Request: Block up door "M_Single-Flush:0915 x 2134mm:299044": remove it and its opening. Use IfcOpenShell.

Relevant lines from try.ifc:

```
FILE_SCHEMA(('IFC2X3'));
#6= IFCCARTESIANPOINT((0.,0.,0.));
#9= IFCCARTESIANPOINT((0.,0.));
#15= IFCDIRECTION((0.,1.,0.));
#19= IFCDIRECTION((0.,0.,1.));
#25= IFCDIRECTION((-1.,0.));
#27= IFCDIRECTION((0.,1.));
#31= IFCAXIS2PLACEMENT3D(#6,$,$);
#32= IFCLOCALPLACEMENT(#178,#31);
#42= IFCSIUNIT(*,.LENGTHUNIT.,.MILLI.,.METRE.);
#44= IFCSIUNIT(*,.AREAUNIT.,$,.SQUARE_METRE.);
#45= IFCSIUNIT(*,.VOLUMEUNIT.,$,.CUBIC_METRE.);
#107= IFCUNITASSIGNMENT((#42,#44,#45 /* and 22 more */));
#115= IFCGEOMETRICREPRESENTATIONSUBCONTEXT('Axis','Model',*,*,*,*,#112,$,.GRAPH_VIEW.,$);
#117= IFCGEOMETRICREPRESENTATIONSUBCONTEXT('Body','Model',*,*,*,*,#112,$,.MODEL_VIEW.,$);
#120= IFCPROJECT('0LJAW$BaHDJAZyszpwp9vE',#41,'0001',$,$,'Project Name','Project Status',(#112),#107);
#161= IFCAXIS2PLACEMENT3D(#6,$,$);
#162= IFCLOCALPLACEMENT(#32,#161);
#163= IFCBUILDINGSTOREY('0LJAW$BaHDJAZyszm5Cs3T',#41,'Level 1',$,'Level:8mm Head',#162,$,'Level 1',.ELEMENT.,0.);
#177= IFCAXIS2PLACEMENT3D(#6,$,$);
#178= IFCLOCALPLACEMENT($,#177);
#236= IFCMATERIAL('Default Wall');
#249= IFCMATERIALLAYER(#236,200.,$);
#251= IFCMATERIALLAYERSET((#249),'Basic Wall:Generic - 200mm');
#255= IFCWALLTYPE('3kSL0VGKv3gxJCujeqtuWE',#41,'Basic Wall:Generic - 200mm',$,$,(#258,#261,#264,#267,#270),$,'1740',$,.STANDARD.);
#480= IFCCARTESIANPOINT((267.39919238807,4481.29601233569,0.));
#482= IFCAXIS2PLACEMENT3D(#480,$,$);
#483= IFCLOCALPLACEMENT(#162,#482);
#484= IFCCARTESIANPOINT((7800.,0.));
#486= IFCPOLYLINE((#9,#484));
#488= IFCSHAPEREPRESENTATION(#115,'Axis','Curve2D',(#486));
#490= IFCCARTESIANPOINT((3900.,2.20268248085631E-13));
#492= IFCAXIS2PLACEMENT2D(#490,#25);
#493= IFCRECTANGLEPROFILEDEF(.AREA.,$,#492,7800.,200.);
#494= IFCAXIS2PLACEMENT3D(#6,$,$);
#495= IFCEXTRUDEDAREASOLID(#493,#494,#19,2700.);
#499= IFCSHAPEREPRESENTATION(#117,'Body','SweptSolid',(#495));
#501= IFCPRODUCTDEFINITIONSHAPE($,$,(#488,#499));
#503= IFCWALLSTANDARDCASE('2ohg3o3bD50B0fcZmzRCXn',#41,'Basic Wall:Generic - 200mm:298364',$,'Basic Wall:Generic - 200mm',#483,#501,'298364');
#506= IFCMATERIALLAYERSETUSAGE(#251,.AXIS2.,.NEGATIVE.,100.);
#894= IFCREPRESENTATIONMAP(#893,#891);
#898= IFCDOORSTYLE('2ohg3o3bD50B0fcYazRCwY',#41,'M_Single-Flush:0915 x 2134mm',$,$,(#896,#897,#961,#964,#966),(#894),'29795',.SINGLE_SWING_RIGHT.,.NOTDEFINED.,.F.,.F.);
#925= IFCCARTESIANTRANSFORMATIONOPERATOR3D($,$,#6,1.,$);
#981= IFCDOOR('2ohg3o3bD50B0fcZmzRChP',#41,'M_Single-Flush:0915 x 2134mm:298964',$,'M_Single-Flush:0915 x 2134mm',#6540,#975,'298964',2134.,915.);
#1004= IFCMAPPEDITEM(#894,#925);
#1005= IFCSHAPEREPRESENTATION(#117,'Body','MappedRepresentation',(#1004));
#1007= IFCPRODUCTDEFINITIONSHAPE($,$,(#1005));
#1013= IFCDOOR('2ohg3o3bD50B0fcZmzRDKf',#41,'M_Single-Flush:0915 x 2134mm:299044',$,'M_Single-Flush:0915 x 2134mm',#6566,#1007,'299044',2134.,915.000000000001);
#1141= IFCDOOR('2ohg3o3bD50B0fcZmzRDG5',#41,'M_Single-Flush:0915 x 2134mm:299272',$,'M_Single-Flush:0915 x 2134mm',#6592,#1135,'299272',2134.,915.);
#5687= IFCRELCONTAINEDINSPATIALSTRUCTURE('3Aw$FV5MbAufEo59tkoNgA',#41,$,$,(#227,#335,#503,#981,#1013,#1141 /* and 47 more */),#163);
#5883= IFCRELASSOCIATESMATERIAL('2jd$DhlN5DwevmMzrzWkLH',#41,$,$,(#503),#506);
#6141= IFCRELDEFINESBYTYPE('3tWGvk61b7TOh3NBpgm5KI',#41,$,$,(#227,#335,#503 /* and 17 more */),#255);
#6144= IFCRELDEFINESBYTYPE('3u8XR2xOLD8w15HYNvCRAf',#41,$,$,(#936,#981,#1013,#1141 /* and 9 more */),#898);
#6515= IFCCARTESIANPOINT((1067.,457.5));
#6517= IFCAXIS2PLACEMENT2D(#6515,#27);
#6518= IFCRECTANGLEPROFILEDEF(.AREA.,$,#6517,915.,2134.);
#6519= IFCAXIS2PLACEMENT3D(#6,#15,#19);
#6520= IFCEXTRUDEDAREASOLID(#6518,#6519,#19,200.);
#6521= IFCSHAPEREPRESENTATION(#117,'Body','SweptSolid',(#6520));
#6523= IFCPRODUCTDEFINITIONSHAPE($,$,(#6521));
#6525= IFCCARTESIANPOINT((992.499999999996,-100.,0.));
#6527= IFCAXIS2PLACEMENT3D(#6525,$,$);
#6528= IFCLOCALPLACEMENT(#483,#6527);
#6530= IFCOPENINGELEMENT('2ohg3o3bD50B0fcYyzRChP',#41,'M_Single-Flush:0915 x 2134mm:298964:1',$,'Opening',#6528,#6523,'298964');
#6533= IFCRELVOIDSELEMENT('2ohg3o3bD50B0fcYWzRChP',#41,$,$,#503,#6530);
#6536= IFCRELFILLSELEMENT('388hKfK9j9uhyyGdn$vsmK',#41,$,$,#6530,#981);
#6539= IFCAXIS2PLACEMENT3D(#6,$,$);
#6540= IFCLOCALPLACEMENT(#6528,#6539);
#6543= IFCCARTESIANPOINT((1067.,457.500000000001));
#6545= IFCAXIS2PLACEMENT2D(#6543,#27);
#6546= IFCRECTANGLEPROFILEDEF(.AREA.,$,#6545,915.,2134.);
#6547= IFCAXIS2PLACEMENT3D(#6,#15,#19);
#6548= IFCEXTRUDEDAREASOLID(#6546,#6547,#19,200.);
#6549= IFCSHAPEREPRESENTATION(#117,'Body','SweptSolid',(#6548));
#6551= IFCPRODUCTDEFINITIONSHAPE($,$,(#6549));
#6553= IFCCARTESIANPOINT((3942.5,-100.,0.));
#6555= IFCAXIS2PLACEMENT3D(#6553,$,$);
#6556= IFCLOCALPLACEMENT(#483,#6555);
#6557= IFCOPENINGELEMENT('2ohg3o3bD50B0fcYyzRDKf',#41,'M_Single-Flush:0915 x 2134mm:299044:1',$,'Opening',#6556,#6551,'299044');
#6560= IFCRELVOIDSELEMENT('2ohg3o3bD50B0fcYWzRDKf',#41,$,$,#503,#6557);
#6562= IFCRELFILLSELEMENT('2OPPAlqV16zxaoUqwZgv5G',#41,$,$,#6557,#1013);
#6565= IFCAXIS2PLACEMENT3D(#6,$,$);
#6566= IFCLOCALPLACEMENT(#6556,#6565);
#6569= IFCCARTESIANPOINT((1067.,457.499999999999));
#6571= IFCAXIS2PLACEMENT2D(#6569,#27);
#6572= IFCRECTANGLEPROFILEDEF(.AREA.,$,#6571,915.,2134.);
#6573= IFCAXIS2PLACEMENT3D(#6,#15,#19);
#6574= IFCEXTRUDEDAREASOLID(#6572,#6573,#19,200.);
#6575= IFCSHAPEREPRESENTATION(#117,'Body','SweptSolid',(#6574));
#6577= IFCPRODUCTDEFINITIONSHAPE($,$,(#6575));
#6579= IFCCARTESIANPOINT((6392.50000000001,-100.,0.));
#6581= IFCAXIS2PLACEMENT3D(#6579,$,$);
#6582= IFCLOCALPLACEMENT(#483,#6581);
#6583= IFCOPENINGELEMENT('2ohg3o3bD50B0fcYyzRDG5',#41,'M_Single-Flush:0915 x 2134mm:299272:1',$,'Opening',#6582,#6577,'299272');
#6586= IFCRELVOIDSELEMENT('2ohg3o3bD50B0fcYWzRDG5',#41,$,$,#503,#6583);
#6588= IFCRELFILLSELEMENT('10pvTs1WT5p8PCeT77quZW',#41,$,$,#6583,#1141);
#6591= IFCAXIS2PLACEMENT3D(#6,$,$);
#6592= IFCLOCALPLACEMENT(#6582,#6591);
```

```python
import ifcopenshell
import ifcopenshell.api.feature
import ifcopenshell.api.root
import ifcopenshell.geom
import ifcopenshell.util.shape

model = ifcopenshell.open("try.ifc")
settings = ifcopenshell.geom.settings()


def volume(element):
    """Net volume in cubic metres, openings subtracted."""
    shape = ifcopenshell.geom.create_shape(settings, element)
    return ifcopenshell.util.shape.get_volume(shape.geometry)


door = model.by_guid("2ohg3o3bD50B0fcZmzRDKf")
opening = door.FillsVoids[0].RelatingOpeningElement
wall = opening.VoidsElements[0].RelatingBuildingElement
before = volume(wall)

ifcopenshell.api.root.remove_product(model, product=door)
ifcopenshell.api.feature.remove_feature(model, feature=opening)

after = volume(wall)

print(f"wall volume {before:.3f} -> {after:.3f} m3")

model.write("try_rev.ifc")
```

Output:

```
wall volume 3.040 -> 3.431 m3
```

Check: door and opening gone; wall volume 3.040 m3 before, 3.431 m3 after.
